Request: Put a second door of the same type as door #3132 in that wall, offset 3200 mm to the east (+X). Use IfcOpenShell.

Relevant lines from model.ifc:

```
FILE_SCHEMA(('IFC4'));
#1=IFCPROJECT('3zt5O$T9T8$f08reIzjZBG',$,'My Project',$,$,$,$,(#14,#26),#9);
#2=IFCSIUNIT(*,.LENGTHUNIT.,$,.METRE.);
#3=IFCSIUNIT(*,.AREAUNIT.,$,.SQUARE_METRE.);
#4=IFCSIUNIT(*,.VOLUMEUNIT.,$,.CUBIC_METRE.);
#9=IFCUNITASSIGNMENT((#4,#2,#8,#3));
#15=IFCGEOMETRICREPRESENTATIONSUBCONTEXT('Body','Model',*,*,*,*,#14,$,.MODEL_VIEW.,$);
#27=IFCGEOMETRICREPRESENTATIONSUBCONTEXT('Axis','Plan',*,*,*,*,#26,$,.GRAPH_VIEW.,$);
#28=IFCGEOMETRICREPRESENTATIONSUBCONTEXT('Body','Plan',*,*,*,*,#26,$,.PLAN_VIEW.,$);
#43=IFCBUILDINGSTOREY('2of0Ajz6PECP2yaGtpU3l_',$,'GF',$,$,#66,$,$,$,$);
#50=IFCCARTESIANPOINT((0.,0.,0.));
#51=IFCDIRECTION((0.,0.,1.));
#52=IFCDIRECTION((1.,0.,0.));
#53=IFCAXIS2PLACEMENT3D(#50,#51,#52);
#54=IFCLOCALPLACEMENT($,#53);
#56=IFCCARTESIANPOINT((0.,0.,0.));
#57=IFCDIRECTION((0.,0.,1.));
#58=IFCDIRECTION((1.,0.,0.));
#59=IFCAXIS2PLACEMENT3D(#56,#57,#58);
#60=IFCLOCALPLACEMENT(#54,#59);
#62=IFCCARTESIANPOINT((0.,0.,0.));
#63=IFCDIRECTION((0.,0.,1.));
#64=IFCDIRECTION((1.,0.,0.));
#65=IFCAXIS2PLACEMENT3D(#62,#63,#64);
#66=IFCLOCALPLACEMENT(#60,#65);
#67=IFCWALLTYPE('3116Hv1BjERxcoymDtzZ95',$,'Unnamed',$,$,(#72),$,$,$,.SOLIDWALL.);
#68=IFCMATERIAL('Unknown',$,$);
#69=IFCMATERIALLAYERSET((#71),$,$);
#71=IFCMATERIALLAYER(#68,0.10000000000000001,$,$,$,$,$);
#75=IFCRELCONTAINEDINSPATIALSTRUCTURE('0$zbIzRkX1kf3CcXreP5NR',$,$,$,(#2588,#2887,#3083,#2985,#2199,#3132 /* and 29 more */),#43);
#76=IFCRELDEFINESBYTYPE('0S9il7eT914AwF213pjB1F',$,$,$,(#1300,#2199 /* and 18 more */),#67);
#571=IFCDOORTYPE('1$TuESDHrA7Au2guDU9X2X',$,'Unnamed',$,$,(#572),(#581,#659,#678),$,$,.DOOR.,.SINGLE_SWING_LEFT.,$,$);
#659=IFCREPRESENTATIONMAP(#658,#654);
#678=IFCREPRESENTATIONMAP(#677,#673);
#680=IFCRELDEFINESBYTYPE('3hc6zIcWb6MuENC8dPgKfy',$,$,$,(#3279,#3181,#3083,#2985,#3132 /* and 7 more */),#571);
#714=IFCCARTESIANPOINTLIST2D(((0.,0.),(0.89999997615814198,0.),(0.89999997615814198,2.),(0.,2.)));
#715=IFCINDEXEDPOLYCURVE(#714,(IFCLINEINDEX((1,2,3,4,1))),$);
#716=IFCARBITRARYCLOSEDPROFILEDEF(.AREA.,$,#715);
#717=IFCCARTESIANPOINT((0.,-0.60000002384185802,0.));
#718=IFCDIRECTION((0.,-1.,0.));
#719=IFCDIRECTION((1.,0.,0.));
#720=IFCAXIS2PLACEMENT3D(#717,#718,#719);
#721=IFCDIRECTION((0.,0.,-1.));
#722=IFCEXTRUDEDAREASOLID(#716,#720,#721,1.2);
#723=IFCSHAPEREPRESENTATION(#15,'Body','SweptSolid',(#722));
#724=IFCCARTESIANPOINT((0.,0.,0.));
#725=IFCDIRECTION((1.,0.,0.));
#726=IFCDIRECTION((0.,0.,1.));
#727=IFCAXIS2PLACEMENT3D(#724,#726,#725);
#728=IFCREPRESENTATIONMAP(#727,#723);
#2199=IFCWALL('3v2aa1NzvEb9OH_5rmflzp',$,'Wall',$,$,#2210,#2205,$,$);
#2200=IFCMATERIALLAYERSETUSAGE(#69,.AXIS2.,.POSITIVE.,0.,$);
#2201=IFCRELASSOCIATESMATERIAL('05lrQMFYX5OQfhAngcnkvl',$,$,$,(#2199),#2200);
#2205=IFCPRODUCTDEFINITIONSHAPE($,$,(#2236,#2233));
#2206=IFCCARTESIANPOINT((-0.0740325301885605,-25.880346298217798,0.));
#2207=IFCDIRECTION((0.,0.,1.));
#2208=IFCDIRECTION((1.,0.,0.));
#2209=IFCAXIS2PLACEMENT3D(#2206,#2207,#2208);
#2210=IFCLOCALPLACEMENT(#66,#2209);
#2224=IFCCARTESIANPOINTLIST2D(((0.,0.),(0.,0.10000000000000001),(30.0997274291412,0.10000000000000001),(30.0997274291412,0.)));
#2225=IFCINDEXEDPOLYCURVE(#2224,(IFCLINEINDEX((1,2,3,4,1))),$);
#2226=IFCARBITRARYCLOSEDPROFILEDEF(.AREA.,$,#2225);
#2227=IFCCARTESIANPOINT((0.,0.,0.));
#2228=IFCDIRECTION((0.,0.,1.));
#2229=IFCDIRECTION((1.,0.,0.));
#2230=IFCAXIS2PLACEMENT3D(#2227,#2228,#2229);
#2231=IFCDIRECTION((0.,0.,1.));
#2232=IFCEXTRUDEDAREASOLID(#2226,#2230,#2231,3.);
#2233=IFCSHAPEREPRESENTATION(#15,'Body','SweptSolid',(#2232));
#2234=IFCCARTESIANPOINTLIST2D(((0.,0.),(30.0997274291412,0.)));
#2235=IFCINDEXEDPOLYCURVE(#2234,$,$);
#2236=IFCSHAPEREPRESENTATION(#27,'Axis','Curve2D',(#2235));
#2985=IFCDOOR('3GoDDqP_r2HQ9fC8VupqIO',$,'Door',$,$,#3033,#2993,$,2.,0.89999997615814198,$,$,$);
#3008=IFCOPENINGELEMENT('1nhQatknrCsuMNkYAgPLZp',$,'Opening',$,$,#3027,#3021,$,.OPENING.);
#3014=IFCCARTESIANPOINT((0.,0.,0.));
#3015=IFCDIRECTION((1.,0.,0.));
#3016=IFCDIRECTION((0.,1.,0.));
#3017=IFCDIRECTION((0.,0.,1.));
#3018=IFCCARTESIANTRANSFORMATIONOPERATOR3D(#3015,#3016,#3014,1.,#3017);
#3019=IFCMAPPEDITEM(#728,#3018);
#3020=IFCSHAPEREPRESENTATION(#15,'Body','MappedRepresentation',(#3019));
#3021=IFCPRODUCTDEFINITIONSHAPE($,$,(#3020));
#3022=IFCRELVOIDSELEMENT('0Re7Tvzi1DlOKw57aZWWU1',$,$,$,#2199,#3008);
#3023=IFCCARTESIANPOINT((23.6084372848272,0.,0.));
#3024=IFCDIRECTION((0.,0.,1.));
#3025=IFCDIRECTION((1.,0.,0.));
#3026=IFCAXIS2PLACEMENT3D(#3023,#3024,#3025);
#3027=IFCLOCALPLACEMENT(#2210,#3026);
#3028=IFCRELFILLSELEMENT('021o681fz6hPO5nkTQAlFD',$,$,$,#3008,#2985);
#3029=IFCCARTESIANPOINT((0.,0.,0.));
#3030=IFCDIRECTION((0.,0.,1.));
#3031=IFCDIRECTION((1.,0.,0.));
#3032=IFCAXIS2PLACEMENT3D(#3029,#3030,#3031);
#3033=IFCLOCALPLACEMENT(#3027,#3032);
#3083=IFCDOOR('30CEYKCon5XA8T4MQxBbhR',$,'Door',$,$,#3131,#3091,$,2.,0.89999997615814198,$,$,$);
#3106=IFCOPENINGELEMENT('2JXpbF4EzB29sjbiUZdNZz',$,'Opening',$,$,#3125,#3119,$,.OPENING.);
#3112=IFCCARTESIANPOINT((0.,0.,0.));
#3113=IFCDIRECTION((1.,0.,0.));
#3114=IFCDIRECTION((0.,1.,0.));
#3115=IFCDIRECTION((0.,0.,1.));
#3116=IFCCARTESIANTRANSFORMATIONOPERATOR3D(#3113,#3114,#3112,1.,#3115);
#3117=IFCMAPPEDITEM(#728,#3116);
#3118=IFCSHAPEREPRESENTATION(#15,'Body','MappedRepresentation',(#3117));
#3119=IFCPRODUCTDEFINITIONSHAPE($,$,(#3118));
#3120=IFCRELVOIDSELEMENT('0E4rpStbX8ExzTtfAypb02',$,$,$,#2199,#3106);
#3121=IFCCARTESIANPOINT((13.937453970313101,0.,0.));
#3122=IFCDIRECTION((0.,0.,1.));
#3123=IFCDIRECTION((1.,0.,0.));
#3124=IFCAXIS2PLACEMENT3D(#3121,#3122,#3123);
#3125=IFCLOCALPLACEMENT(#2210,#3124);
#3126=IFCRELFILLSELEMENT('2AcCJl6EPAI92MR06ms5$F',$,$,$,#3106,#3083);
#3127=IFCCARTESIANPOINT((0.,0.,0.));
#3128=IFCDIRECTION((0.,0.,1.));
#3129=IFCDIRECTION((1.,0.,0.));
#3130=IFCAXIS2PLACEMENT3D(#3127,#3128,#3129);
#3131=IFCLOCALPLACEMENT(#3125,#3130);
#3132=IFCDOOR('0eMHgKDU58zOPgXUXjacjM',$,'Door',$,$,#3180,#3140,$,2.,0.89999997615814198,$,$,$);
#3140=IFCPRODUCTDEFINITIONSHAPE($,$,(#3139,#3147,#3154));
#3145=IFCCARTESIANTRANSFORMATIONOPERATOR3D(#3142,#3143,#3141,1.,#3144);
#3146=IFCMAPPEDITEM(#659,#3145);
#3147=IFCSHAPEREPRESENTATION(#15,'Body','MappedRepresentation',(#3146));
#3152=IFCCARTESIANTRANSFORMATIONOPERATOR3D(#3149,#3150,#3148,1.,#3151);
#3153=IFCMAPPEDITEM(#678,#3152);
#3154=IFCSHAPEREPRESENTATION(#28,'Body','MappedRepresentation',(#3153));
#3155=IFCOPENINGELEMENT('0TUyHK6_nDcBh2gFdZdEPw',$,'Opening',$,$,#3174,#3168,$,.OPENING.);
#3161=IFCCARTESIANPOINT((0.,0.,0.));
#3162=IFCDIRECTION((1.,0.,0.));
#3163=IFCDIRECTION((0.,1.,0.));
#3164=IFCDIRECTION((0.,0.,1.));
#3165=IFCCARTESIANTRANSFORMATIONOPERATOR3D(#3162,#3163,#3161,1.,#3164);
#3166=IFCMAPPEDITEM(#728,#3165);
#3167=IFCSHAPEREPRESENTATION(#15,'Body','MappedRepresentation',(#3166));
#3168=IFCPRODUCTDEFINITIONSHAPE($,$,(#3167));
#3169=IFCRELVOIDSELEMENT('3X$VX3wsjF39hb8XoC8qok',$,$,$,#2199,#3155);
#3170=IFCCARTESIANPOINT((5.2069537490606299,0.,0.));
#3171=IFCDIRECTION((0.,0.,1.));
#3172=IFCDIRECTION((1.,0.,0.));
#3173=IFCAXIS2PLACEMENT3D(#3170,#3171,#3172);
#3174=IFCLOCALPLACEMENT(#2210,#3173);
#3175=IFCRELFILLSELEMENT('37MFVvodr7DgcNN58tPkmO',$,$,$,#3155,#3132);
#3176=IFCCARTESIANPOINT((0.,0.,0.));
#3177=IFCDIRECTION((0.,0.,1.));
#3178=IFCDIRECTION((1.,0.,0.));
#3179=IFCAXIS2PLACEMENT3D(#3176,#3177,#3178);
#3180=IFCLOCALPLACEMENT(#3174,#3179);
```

```python
import ifcopenshell
import ifcopenshell.api.feature
import ifcopenshell.api.geometry
import ifcopenshell.api.root
import ifcopenshell.geom
import ifcopenshell.util.element
import ifcopenshell.util.placement
import ifcopenshell.util.shape
import ifcopenshell.util.unit

model = ifcopenshell.open("model.ifc")
unit_scale = ifcopenshell.util.unit.calculate_unit_scale(model)
settings = ifcopenshell.geom.settings()


def volume(element):
    """Net volume in cubic metres, openings subtracted."""
    shape = ifcopenshell.geom.create_shape(settings, element)
    return ifcopenshell.util.shape.get_volume(shape.geometry)


door = model.by_guid("0eMHgKDU58zOPgXUXjacjM")
opening = door.FillsVoids[0].RelatingOpeningElement
wall = opening.VoidsElements[0].RelatingBuildingElement
before = volume(wall)
shift = ifcopenshell.util.placement.get_local_placement(wall.ObjectPlacement)[:3, 0] * 3.2 / unit_scale

# copy_class copies the void relationship, type, container and properties, but no geometry.
new_opening = ifcopenshell.api.root.copy_class(model, product=opening)
new_opening.Representation = ifcopenshell.util.element.copy_deep(
    model, opening.Representation, exclude=["IfcGeometricRepresentationContext", "IfcRepresentationMap"]
)
new_door = ifcopenshell.api.root.copy_class(model, product=door)
new_door.Representation = ifcopenshell.util.element.copy_deep(
    model, door.Representation, exclude=["IfcGeometricRepresentationContext", "IfcRepresentationMap"]
)
ifcopenshell.api.feature.add_filling(model, opening=new_opening, element=new_door)

for old, new in ((opening, new_opening), (door, new_door)):
    matrix = ifcopenshell.util.placement.get_local_placement(old.ObjectPlacement)
    matrix[:3, 3] += shift
    ifcopenshell.api.geometry.edit_object_placement(model, product=new, matrix=matrix, is_si=False)

after = volume(wall)

print(f"wall volume {before:.3f} -> {after:.3f} m3")

model.write("model_edited.ifc")
```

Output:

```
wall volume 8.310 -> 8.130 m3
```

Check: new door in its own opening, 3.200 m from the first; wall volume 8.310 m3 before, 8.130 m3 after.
